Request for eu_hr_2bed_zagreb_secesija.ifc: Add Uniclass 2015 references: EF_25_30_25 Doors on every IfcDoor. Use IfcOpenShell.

First a look at what the model holds.

```python
import ifcopenshell

model = ifcopenshell.open("eu_hr_2bed_zagreb_secesija.ifc")
print(model.schema)
print("classifications:", [c.Name for c in model.by_type("IfcClassification")])
for ifc_class in ("IfcDoor", "IfcRoof", "IfcStair", "IfcWall", "IfcWindow"):
    print(ifc_class, len(model.by_type(ifc_class)))
```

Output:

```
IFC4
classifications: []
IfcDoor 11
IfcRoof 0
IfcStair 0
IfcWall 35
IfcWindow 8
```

```python
import ifcopenshell
import ifcopenshell.api.classification

model = ifcopenshell.open("eu_hr_2bed_zagreb_secesija.ifc")

system = ifcopenshell.api.classification.add_classification(model, classification="Uniclass 2015")

codes = {
    "IfcDoor": ("EF_25_30_25", "Doors"),
}
for ifc_class, (code, name) in codes.items():
    products = model.by_type(ifc_class)
    ifcopenshell.api.classification.add_reference(
        model, products=products, classification=system, identification=code, name=name
    )
    print(code, len(products))

model.write("eu_hr_2bed_zagreb_secesija_v2.ifc")
```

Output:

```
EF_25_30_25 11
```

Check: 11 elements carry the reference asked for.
